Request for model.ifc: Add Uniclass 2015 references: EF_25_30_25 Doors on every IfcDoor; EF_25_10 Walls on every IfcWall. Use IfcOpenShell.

First a look at what the model holds.

```python
import ifcopenshell

model = ifcopenshell.open("model.ifc")
print(model.schema)
print("classifications:", [c.Name for c in model.by_type("IfcClassification")])
for ifc_class in ("IfcDoor", "IfcRoof", "IfcStair", "IfcWall", "IfcWindow"):
    print(ifc_class, len(model.by_type(ifc_class)))
```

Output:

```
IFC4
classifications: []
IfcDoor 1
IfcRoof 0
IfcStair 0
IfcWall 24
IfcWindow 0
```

```python
import ifcopenshell
import ifcopenshell.api.classification

model = ifcopenshell.open("model.ifc")

system = ifcopenshell.api.classification.add_classification(model, classification="Uniclass 2015")

codes = {
    "IfcDoor": ("EF_25_30_25", "Doors"),
    "IfcWall": ("EF_25_10", "Walls"),
}
for ifc_class, (code, name) in codes.items():
    products = model.by_type(ifc_class)
    ifcopenshell.api.classification.add_reference(
        model, products=products, classification=system, identification=code, name=name
    )
    print(code, len(products))

model.write("model_edited.ifc")
```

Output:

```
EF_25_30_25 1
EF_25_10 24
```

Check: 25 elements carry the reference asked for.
